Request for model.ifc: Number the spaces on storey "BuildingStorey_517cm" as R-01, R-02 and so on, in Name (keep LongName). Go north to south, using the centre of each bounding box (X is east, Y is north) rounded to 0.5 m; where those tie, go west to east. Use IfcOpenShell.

First a look at what the model holds.

```python
import ifcopenshell
import ifcopenshell.util.element
import ifcopenshell.util.placement

model = ifcopenshell.open("model.ifc")
print(model.schema)
storey = next(s for s in model.by_type("IfcBuildingStorey") if s.Name == "BuildingStorey_517cm")
spaces = [e for e in ifcopenshell.util.element.get_decomposition(storey) if e.is_a("IfcSpace")]
for e in sorted(spaces, key=lambda e: e.id()):
    origin = ifcopenshell.util.placement.get_local_placement(e.ObjectPlacement)[:3, 3]
    print(e.id(), e.Name, e.LongName, origin.round(2) + 0.0, sep=" | ")
```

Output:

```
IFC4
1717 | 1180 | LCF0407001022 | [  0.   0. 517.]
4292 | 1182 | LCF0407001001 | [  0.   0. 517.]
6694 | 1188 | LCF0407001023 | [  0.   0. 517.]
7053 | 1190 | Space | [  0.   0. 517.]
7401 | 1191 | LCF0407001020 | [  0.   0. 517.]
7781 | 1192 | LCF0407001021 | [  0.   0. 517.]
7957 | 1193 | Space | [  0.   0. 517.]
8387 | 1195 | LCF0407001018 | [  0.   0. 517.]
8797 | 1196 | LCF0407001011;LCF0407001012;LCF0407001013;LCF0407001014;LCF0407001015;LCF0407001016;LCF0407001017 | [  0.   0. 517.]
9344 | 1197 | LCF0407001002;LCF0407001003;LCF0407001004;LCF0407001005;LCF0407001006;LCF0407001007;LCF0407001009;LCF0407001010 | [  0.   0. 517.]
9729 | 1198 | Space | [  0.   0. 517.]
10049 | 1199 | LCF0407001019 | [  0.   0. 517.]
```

```python
import ifcopenshell
import ifcopenshell.geom
import ifcopenshell.util.element
import ifcopenshell.util.shape

model = ifcopenshell.open("model.ifc")
settings = ifcopenshell.geom.settings()
settings.set("use-world-coords", True)


def centre(element):
    shape = ifcopenshell.geom.create_shape(settings, element)
    return ifcopenshell.util.shape.get_bbox_centroid(shape.geometry)


storey = next(s for s in model.by_type("IfcBuildingStorey") if s.Name == "BuildingStorey_517cm")
spaces = [e for e in ifcopenshell.util.element.get_decomposition(storey) if e.is_a("IfcSpace")]

# Insertion points can sit at a corner or the storey origin, so sort by the geometry (in metres).
centres = {e: centre(e) for e in spaces}
spaces.sort(key=lambda e: (-round(centres[e][1] / 0.5), centres[e][0]))

for i, e in enumerate(spaces, start=1):
    number = f"R-{i:02d}"
    e.Name = number
    print(e.id(), number)

model.write("model_v2.ifc")
```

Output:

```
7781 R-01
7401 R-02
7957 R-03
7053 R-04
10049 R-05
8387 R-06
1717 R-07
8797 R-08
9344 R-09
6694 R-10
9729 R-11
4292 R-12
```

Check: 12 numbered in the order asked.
